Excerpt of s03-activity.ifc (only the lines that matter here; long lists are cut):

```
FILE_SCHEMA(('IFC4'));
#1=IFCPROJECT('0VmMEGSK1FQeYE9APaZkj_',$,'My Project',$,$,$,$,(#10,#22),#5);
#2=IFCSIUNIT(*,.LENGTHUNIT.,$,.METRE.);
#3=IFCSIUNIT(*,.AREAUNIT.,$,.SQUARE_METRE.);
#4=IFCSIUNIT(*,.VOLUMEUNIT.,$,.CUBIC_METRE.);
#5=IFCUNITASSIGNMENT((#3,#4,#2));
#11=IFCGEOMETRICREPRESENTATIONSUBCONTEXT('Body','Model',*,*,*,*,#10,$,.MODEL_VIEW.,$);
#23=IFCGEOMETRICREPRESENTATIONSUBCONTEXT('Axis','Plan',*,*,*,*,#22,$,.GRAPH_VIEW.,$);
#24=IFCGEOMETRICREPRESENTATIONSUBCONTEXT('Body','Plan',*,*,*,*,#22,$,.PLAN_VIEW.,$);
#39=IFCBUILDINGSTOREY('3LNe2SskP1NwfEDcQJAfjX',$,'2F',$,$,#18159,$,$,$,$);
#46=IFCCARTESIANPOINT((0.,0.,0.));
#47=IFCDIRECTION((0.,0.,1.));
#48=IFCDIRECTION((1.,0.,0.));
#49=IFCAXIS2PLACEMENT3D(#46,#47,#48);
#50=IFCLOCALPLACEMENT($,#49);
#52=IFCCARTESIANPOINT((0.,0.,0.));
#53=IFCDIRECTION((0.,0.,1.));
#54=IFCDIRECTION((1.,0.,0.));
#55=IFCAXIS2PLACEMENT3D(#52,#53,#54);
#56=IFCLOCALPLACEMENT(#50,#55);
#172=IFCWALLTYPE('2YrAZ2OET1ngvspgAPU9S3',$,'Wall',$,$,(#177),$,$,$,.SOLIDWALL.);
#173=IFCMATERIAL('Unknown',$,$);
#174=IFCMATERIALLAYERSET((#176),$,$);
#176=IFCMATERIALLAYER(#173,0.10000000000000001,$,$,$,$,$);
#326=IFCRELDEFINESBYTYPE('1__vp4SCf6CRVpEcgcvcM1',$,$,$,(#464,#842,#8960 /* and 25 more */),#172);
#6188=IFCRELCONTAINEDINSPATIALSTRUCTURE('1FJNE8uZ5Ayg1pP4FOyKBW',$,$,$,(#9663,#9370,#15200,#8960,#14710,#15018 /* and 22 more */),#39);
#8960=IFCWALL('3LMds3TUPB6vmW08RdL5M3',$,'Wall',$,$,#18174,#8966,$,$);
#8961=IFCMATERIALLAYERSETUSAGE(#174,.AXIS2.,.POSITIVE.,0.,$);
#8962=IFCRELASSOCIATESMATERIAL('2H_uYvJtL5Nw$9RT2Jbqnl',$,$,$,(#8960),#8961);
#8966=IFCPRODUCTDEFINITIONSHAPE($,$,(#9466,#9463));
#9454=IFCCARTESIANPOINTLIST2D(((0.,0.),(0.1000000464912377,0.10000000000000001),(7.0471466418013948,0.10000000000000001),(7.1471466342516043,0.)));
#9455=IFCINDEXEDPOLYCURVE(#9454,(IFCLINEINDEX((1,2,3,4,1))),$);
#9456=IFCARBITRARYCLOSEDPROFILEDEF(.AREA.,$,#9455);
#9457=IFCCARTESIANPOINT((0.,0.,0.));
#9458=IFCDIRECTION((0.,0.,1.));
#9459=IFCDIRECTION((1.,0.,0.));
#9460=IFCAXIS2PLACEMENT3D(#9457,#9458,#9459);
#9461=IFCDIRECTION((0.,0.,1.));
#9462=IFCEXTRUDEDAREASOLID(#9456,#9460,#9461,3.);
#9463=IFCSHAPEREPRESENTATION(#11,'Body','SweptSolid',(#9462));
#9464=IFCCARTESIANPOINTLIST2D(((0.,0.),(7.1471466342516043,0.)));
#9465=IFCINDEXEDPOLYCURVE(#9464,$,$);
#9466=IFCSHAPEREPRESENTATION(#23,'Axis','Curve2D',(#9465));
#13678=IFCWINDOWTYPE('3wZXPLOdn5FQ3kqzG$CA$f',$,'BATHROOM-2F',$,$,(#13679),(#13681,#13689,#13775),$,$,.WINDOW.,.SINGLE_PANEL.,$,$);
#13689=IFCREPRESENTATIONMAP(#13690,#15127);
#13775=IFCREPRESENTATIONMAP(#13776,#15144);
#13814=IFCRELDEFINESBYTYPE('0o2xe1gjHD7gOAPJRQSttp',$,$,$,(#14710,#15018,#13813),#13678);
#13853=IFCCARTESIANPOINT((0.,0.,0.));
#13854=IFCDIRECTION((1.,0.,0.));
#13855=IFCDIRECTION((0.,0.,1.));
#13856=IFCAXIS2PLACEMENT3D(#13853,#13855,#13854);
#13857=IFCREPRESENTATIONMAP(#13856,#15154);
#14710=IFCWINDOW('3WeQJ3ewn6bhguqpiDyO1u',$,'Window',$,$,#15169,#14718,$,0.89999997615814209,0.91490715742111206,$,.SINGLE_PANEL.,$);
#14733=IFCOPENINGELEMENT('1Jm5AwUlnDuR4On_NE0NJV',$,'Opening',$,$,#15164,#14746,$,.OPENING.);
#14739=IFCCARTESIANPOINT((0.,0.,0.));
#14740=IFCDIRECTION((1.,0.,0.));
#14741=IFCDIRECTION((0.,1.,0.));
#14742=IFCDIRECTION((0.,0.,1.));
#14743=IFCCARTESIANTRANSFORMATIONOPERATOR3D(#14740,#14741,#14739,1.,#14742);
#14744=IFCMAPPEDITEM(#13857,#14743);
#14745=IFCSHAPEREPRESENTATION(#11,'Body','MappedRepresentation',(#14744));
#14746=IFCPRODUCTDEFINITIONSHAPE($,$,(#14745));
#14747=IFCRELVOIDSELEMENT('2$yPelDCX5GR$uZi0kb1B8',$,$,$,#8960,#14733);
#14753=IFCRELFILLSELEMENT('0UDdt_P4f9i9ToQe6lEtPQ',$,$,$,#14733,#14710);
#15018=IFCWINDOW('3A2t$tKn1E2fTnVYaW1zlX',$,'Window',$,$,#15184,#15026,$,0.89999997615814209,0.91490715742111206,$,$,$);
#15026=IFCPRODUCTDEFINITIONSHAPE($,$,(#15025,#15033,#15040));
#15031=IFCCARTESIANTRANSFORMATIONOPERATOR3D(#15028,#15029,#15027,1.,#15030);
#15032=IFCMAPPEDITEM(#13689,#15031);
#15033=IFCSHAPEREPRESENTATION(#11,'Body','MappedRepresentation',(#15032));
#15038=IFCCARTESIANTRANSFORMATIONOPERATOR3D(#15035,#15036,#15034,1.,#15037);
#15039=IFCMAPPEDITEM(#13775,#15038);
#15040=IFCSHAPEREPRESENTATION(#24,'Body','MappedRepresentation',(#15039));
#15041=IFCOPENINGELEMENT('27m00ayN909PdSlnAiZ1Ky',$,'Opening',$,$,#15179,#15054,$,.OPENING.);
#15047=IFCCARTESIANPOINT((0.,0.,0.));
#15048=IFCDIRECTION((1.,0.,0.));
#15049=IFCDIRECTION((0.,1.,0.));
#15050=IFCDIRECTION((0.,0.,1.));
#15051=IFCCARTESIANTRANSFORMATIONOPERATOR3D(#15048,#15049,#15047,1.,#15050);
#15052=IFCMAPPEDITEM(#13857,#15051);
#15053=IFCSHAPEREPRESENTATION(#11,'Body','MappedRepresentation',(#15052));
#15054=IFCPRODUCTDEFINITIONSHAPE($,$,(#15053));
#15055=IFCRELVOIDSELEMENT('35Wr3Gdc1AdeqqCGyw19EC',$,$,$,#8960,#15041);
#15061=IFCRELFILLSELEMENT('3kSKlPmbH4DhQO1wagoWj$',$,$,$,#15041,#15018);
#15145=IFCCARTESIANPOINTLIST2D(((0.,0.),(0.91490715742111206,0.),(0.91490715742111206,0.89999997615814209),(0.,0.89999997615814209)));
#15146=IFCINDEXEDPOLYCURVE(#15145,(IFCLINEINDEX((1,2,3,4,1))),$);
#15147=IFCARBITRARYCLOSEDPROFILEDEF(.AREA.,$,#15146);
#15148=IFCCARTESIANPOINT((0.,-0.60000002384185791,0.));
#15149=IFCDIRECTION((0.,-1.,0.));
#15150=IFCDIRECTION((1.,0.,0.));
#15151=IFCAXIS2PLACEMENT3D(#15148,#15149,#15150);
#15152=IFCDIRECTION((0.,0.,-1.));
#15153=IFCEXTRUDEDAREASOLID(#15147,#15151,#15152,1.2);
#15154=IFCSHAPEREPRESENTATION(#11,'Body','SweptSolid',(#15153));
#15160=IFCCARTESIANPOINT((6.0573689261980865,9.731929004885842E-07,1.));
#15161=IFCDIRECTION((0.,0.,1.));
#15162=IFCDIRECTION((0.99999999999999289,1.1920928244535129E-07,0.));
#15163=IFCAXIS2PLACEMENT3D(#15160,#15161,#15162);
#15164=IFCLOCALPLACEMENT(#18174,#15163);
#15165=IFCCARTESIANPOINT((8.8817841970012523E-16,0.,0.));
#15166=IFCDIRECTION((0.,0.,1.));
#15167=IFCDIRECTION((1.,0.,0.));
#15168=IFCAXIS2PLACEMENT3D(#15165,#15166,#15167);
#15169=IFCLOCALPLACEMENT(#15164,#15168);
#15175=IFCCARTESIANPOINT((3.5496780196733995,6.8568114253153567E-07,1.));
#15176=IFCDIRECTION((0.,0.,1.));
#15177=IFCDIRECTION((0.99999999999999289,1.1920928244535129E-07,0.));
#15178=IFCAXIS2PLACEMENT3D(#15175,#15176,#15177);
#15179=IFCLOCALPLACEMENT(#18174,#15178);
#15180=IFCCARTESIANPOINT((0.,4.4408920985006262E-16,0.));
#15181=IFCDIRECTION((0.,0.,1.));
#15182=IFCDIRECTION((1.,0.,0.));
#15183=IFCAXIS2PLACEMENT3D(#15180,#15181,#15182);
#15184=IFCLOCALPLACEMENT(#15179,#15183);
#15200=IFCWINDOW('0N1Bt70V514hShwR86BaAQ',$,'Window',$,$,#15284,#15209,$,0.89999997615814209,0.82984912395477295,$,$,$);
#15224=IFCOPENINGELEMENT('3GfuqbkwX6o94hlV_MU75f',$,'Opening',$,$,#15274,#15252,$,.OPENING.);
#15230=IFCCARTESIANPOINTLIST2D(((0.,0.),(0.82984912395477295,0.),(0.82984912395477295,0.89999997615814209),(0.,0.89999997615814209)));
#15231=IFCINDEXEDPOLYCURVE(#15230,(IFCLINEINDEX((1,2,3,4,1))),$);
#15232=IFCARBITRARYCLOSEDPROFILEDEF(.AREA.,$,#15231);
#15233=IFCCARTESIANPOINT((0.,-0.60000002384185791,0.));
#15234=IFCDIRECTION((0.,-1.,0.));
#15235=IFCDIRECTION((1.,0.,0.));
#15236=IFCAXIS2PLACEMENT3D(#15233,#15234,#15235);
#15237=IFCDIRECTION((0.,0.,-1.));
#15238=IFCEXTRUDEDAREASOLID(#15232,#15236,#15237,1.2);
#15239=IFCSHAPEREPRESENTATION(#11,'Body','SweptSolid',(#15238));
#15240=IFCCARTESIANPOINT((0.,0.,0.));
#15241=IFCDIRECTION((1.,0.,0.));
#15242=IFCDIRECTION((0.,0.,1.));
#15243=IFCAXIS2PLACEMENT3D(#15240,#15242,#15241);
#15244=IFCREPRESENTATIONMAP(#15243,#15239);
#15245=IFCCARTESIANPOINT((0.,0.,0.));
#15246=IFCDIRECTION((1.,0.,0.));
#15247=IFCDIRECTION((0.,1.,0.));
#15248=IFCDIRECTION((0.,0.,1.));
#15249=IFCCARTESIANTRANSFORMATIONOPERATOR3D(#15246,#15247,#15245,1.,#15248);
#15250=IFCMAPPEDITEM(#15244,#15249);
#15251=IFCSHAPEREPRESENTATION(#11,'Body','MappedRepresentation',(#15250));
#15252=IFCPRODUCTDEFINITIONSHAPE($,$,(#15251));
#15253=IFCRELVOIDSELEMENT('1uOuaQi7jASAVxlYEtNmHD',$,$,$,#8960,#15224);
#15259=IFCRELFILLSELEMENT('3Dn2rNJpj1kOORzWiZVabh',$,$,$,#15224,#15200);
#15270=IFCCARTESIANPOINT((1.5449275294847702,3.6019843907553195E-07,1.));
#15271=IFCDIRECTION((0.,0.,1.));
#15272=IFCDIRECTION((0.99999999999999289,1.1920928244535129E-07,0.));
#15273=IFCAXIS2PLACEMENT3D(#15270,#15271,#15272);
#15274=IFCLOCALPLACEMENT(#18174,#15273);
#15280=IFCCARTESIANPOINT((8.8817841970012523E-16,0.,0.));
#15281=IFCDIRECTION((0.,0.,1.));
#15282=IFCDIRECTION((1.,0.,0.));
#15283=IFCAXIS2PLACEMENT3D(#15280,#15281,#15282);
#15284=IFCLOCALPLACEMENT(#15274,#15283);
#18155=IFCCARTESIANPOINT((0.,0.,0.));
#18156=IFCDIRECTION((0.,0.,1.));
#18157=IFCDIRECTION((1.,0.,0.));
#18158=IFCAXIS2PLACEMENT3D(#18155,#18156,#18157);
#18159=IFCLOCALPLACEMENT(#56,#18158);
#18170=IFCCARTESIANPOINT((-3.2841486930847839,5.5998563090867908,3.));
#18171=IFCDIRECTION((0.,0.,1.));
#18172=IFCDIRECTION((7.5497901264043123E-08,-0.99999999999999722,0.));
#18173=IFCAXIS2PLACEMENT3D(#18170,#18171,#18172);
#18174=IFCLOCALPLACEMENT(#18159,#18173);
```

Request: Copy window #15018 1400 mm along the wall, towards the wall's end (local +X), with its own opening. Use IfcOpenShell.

```python
import ifcopenshell
import ifcopenshell.api.feature
import ifcopenshell.api.geometry
import ifcopenshell.api.root
import ifcopenshell.geom
import ifcopenshell.util.element
import ifcopenshell.util.placement
import ifcopenshell.util.shape
import ifcopenshell.util.unit

model = ifcopenshell.open("s03-activity.ifc")
unit_scale = ifcopenshell.util.unit.calculate_unit_scale(model)
settings = ifcopenshell.geom.settings()


def volume(element):
    """Net volume in cubic metres, openings subtracted."""
    shape = ifcopenshell.geom.create_shape(settings, element)
    return ifcopenshell.util.shape.get_volume(shape.geometry)


window = model.by_guid("3A2t$tKn1E2fTnVYaW1zlX")
opening = window.FillsVoids[0].RelatingOpeningElement
wall = opening.VoidsElements[0].RelatingBuildingElement
before = volume(wall)
shift = ifcopenshell.util.placement.get_local_placement(wall.ObjectPlacement)[:3, 0] * 1.4 / unit_scale

# copy_class copies the void relationship, type, container and properties, but no geometry.
new_opening = ifcopenshell.api.root.copy_class(model, product=opening)
new_opening.Representation = ifcopenshell.util.element.copy_deep(
    model, opening.Representation, exclude=["IfcGeometricRepresentationContext", "IfcRepresentationMap"]
)
new_window = ifcopenshell.api.root.copy_class(model, product=window)
new_window.Representation = ifcopenshell.util.element.copy_deep(
    model, window.Representation, exclude=["IfcGeometricRepresentationContext", "IfcRepresentationMap"]
)
ifcopenshell.api.feature.add_filling(model, opening=new_opening, element=new_window)

for old, new in ((opening, new_opening), (window, new_window)):
    matrix = ifcopenshell.util.placement.get_local_placement(old.ObjectPlacement)
    matrix[:3, 3] += shift
    ifcopenshell.api.geometry.edit_object_placement(model, product=new, matrix=matrix, is_si=False)

after = volume(wall)

print(f"wall volume {before:.3f} -> {after:.3f} m3")

model.write("s03-activity_rev.ifc")
```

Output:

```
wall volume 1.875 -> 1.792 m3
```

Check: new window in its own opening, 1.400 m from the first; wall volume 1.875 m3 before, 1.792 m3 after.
